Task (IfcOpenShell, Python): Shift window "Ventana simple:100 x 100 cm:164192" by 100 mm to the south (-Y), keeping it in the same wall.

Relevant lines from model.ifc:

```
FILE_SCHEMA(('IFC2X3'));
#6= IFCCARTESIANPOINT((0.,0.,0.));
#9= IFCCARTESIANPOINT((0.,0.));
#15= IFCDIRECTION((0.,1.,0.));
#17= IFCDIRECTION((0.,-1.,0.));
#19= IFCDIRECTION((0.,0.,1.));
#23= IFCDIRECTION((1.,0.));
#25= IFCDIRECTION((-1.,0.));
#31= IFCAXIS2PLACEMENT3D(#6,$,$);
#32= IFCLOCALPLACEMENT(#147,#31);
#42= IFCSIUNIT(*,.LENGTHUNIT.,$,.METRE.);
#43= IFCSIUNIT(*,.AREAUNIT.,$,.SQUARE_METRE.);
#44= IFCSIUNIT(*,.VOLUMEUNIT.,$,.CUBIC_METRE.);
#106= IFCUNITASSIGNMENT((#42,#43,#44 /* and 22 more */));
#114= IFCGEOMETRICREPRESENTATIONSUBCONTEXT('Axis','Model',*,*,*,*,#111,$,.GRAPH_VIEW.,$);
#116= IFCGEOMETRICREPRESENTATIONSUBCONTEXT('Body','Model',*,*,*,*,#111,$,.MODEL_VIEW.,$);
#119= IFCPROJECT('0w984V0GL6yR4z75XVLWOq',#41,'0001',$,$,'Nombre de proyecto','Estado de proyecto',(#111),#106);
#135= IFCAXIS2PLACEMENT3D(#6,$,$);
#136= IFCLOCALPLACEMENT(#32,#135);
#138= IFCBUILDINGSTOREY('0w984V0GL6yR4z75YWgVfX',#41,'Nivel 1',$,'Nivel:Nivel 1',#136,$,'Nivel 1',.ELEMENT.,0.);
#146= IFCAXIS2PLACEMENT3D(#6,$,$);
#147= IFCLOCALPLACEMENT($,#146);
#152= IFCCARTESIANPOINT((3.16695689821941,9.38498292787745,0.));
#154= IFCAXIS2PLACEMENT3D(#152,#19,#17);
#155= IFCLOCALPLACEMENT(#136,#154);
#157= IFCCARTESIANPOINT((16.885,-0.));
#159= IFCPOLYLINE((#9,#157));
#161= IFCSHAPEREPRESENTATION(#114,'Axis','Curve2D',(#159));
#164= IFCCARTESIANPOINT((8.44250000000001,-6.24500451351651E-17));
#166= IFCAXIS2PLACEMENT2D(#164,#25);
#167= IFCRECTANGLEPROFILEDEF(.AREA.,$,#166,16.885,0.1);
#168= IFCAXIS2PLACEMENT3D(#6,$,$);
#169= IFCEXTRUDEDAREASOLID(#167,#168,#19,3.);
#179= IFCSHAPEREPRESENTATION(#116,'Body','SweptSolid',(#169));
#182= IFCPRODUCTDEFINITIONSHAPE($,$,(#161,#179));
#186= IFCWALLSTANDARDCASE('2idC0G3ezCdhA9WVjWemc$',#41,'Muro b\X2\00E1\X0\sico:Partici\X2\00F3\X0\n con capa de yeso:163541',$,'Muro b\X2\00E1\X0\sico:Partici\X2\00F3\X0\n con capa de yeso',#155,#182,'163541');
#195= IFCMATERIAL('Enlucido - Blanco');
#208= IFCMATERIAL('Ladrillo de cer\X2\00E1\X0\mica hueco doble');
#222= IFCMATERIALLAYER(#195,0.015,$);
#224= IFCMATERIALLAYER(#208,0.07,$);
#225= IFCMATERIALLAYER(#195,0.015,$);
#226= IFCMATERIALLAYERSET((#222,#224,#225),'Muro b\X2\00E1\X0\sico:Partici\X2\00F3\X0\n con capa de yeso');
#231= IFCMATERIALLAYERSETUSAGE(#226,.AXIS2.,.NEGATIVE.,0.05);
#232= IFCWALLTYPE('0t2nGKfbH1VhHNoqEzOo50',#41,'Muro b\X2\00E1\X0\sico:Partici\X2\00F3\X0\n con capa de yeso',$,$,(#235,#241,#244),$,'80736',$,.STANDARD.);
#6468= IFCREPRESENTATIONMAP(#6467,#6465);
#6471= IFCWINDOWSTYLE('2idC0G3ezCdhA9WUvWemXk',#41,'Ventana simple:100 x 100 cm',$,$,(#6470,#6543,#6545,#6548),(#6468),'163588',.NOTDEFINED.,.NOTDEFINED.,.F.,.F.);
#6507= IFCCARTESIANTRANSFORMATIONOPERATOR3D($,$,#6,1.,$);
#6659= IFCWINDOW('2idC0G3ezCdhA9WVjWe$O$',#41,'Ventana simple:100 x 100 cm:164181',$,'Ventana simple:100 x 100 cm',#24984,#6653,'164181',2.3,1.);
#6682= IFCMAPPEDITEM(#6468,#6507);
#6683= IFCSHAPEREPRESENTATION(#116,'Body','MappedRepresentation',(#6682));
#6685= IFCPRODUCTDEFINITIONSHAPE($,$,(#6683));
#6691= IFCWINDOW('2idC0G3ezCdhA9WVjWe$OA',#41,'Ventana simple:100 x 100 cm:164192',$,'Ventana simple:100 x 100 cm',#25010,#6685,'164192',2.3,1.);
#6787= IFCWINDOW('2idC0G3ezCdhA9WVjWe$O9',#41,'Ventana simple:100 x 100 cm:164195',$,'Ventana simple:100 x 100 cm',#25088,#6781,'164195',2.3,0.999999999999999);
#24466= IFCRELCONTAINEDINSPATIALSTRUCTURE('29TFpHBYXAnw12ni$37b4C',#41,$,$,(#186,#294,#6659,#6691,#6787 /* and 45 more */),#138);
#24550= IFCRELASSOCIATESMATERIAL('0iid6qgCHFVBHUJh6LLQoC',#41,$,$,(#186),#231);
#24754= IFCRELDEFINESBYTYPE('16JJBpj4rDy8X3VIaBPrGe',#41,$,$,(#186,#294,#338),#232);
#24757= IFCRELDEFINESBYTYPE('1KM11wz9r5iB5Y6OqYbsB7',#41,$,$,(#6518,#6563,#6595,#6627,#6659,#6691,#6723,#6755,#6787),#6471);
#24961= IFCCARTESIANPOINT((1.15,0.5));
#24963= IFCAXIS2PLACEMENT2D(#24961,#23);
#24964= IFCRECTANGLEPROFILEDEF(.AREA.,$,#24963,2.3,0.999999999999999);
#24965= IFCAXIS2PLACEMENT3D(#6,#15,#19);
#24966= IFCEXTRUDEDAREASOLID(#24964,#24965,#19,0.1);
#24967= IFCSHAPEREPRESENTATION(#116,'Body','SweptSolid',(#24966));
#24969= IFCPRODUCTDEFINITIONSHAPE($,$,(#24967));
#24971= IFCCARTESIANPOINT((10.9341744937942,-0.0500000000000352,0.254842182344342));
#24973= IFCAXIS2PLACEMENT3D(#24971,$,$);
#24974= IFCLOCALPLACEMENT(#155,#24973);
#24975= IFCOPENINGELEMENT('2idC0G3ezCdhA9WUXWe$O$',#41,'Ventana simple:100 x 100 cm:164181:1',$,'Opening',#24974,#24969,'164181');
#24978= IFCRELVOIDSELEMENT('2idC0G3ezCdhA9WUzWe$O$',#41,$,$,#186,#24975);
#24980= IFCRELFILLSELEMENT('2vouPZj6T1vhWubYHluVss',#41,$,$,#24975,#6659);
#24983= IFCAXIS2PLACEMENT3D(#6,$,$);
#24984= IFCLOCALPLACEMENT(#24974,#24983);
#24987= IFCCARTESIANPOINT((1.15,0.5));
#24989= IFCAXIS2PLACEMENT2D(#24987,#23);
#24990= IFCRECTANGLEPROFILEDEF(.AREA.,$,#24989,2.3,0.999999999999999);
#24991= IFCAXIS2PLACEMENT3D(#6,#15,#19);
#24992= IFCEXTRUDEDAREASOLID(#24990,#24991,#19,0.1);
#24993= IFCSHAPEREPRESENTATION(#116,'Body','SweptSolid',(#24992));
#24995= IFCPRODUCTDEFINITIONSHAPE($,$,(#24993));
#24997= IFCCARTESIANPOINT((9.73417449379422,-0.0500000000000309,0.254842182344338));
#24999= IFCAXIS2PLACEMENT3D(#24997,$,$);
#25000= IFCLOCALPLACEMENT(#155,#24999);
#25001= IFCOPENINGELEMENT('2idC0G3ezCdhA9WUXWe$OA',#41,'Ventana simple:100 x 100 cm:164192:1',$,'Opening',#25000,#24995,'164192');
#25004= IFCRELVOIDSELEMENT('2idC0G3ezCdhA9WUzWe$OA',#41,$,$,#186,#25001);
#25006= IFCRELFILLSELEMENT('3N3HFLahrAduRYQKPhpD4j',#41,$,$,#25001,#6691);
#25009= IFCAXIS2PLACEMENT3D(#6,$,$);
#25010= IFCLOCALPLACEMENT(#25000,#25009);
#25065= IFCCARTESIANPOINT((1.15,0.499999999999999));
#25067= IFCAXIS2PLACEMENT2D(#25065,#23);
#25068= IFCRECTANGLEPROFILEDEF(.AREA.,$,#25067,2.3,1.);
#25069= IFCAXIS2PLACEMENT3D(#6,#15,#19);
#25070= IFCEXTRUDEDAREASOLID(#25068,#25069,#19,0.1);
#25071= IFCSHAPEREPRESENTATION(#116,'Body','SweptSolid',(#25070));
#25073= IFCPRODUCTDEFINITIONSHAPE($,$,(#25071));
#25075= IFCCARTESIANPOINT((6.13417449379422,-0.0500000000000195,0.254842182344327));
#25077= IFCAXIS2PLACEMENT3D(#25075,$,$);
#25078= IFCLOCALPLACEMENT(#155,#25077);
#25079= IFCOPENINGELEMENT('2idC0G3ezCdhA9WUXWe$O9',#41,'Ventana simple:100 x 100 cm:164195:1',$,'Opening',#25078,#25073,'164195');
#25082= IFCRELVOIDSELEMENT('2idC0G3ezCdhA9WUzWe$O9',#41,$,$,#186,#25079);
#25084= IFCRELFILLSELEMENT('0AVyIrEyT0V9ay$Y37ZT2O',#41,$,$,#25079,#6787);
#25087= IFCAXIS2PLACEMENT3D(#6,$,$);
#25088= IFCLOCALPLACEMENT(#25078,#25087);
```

```python
import ifcopenshell
import ifcopenshell.api.geometry
import ifcopenshell.util.placement
import ifcopenshell.util.unit

model = ifcopenshell.open("model.ifc")
unit_scale = ifcopenshell.util.unit.calculate_unit_scale(model)

window = model.by_guid("2idC0G3ezCdhA9WVjWe$OA")
opening = window.FillsVoids[0].RelatingOpeningElement
wall = opening.VoidsElements[0].RelatingBuildingElement

wall_matrix = ifcopenshell.util.placement.get_local_placement(wall.ObjectPlacement)
shift = wall_matrix[:3, 0] * 0.1 / unit_scale
before = ifcopenshell.util.placement.get_local_placement(window.ObjectPlacement)[:3, 3].copy()

# The window is placed relative to its opening, so it follows when the opening moves.
matrix = ifcopenshell.util.placement.get_local_placement(opening.ObjectPlacement)
matrix[:3, 3] += shift
ifcopenshell.api.geometry.edit_object_placement(
    model, product=opening, matrix=matrix, is_si=False, should_transform_children=True
)

after = ifcopenshell.util.placement.get_local_placement(window.ObjectPlacement)[:3, 3]
print("window moved by", (after - before).round(3) + 0.0)

model.write("model_updated.ifc")
```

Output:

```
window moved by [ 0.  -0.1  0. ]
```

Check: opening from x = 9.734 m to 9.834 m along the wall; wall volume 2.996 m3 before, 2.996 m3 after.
